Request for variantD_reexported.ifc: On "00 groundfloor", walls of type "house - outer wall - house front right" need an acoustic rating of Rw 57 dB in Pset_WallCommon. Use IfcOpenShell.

First a look at what the model holds.

```python
import ifcopenshell
import ifcopenshell.util.element

model = ifcopenshell.open("variantD_reexported.ifc")
print(model.schema)
storey = next(s for s in model.by_type("IfcBuildingStorey") if s.Name == "00 groundfloor")
walls = [e for e in ifcopenshell.util.element.get_decomposition(storey) if e.is_a("IfcWall")]
seen = {}
for e in walls:
    element_type = ifcopenshell.util.element.get_type(e)
    key = (element_type.Name if element_type != e and element_type else None, ifcopenshell.util.element.get_pset(e, "Pset_WallCommon", "AcousticRating"))
    seen[key] = seen.get(key, 0) + 1
for (name, value), count in sorted(seen.items(), key=str):
    print(count, "x", name, "|", value)
```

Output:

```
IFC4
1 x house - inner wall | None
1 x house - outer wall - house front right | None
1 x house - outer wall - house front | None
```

```python
import ifcopenshell
import ifcopenshell.api.pset
import ifcopenshell.util.element

model = ifcopenshell.open("variantD_reexported.ifc")

storey = next(s for s in model.by_type("IfcBuildingStorey") if s.Name == "00 groundfloor")
walls = [e for e in ifcopenshell.util.element.get_decomposition(storey) if e.is_a("IfcWall")]

count = 0
for e in walls:
    element_type = ifcopenshell.util.element.get_type(e)
    if element_type in (None, e) or element_type.Name != "house - outer wall - house front right":
        continue
    # add_pset returns the element's existing set when there is one.
    pset = ifcopenshell.api.pset.add_pset(model, product=e, name="Pset_WallCommon")
    ifcopenshell.api.pset.edit_pset(model, pset=pset, properties={"AcousticRating": "Rw 57 dB"})
    count += 1

print(count, "walls updated")

model.write("variantD_reexported-out.ifc")
```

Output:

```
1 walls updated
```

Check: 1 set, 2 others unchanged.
